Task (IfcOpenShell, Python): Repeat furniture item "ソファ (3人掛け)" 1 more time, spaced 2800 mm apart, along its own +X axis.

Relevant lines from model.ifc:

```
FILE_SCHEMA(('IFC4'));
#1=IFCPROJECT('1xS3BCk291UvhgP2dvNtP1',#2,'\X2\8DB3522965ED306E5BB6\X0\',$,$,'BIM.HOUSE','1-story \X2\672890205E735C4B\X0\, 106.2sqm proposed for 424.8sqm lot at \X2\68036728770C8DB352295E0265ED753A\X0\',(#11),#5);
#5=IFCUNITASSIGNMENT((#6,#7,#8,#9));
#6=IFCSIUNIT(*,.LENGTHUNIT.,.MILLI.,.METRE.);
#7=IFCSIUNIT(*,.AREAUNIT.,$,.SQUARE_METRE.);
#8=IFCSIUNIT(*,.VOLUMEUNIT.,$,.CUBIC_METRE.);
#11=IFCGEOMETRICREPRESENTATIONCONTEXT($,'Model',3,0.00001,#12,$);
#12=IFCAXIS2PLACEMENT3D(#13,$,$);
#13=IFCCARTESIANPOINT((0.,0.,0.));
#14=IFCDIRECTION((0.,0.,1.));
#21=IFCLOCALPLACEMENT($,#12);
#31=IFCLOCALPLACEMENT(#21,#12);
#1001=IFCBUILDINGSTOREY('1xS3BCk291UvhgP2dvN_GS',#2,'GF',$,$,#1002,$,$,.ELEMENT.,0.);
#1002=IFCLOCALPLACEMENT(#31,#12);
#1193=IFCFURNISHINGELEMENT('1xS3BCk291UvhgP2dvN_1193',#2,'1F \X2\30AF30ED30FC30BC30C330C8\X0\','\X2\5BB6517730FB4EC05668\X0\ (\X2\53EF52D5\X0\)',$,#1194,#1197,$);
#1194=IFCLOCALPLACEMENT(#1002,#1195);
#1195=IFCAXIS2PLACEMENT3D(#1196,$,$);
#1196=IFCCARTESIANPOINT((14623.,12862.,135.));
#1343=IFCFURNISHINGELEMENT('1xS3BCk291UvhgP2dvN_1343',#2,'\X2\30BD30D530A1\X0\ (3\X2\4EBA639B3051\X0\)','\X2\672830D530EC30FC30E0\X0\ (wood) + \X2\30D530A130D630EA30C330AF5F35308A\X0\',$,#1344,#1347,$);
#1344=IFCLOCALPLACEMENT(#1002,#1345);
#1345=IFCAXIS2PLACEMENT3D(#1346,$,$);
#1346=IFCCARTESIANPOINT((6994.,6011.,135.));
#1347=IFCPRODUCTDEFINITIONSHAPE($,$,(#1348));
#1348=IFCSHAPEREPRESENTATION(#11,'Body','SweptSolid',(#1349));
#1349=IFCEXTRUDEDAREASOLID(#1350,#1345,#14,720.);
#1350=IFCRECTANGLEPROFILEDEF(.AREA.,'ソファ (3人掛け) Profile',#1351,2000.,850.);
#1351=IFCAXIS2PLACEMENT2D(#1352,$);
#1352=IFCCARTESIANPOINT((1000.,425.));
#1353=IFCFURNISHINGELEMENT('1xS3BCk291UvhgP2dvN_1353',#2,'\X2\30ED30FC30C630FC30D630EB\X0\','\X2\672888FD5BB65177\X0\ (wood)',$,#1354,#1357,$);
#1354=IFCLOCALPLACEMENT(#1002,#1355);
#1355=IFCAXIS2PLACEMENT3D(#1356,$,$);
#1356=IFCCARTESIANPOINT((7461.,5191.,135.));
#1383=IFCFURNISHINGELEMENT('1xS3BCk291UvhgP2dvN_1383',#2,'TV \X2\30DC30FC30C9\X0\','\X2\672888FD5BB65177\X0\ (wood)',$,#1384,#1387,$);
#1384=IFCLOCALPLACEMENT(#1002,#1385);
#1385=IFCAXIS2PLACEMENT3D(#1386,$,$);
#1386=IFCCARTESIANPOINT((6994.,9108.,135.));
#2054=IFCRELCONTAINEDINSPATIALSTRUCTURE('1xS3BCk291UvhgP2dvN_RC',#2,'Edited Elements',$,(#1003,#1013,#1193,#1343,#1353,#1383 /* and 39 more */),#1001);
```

```python
import ifcopenshell
import ifcopenshell.api.geometry
import ifcopenshell.api.root
import ifcopenshell.util.element
import ifcopenshell.util.placement
import ifcopenshell.util.unit

model = ifcopenshell.open("model.ifc")
unit_scale = ifcopenshell.util.unit.calculate_unit_scale(model)


def reuse_history(source, copy):
    """copy_class also copies each property set's owner history, people and application; keep the originals."""
    for rel in copy.IsDefinedBy:
        if rel.is_a("IfcRelDefinesByProperties") and (history := rel.RelatingPropertyDefinition.OwnerHistory):
            rel.RelatingPropertyDefinition.OwnerHistory = source.OwnerHistory
            ifcopenshell.util.element.remove_deep2(model, history)


source = model.by_guid("1xS3BCk291UvhgP2dvN_1343")
base = ifcopenshell.util.placement.get_local_placement(source.ObjectPlacement)
step = base[:3, 0] * 2.8 / unit_scale

for i in range(1, 2):
    copy = ifcopenshell.api.root.copy_class(model, product=source)
    copy.Representation = ifcopenshell.util.element.copy_deep(
        model, source.Representation, exclude=["IfcGeometricRepresentationContext", "IfcRepresentationMap"]
    )
    reuse_history(source, copy)
    matrix = base.copy()
    matrix[:3, 3] += i * step
    print("added at", matrix[:3, 3].round(3) + 0.0)
    ifcopenshell.api.geometry.edit_object_placement(model, product=copy, matrix=matrix, is_si=False)

model.write("model_edited.ifc")
```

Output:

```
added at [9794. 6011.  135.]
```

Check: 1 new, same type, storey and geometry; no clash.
